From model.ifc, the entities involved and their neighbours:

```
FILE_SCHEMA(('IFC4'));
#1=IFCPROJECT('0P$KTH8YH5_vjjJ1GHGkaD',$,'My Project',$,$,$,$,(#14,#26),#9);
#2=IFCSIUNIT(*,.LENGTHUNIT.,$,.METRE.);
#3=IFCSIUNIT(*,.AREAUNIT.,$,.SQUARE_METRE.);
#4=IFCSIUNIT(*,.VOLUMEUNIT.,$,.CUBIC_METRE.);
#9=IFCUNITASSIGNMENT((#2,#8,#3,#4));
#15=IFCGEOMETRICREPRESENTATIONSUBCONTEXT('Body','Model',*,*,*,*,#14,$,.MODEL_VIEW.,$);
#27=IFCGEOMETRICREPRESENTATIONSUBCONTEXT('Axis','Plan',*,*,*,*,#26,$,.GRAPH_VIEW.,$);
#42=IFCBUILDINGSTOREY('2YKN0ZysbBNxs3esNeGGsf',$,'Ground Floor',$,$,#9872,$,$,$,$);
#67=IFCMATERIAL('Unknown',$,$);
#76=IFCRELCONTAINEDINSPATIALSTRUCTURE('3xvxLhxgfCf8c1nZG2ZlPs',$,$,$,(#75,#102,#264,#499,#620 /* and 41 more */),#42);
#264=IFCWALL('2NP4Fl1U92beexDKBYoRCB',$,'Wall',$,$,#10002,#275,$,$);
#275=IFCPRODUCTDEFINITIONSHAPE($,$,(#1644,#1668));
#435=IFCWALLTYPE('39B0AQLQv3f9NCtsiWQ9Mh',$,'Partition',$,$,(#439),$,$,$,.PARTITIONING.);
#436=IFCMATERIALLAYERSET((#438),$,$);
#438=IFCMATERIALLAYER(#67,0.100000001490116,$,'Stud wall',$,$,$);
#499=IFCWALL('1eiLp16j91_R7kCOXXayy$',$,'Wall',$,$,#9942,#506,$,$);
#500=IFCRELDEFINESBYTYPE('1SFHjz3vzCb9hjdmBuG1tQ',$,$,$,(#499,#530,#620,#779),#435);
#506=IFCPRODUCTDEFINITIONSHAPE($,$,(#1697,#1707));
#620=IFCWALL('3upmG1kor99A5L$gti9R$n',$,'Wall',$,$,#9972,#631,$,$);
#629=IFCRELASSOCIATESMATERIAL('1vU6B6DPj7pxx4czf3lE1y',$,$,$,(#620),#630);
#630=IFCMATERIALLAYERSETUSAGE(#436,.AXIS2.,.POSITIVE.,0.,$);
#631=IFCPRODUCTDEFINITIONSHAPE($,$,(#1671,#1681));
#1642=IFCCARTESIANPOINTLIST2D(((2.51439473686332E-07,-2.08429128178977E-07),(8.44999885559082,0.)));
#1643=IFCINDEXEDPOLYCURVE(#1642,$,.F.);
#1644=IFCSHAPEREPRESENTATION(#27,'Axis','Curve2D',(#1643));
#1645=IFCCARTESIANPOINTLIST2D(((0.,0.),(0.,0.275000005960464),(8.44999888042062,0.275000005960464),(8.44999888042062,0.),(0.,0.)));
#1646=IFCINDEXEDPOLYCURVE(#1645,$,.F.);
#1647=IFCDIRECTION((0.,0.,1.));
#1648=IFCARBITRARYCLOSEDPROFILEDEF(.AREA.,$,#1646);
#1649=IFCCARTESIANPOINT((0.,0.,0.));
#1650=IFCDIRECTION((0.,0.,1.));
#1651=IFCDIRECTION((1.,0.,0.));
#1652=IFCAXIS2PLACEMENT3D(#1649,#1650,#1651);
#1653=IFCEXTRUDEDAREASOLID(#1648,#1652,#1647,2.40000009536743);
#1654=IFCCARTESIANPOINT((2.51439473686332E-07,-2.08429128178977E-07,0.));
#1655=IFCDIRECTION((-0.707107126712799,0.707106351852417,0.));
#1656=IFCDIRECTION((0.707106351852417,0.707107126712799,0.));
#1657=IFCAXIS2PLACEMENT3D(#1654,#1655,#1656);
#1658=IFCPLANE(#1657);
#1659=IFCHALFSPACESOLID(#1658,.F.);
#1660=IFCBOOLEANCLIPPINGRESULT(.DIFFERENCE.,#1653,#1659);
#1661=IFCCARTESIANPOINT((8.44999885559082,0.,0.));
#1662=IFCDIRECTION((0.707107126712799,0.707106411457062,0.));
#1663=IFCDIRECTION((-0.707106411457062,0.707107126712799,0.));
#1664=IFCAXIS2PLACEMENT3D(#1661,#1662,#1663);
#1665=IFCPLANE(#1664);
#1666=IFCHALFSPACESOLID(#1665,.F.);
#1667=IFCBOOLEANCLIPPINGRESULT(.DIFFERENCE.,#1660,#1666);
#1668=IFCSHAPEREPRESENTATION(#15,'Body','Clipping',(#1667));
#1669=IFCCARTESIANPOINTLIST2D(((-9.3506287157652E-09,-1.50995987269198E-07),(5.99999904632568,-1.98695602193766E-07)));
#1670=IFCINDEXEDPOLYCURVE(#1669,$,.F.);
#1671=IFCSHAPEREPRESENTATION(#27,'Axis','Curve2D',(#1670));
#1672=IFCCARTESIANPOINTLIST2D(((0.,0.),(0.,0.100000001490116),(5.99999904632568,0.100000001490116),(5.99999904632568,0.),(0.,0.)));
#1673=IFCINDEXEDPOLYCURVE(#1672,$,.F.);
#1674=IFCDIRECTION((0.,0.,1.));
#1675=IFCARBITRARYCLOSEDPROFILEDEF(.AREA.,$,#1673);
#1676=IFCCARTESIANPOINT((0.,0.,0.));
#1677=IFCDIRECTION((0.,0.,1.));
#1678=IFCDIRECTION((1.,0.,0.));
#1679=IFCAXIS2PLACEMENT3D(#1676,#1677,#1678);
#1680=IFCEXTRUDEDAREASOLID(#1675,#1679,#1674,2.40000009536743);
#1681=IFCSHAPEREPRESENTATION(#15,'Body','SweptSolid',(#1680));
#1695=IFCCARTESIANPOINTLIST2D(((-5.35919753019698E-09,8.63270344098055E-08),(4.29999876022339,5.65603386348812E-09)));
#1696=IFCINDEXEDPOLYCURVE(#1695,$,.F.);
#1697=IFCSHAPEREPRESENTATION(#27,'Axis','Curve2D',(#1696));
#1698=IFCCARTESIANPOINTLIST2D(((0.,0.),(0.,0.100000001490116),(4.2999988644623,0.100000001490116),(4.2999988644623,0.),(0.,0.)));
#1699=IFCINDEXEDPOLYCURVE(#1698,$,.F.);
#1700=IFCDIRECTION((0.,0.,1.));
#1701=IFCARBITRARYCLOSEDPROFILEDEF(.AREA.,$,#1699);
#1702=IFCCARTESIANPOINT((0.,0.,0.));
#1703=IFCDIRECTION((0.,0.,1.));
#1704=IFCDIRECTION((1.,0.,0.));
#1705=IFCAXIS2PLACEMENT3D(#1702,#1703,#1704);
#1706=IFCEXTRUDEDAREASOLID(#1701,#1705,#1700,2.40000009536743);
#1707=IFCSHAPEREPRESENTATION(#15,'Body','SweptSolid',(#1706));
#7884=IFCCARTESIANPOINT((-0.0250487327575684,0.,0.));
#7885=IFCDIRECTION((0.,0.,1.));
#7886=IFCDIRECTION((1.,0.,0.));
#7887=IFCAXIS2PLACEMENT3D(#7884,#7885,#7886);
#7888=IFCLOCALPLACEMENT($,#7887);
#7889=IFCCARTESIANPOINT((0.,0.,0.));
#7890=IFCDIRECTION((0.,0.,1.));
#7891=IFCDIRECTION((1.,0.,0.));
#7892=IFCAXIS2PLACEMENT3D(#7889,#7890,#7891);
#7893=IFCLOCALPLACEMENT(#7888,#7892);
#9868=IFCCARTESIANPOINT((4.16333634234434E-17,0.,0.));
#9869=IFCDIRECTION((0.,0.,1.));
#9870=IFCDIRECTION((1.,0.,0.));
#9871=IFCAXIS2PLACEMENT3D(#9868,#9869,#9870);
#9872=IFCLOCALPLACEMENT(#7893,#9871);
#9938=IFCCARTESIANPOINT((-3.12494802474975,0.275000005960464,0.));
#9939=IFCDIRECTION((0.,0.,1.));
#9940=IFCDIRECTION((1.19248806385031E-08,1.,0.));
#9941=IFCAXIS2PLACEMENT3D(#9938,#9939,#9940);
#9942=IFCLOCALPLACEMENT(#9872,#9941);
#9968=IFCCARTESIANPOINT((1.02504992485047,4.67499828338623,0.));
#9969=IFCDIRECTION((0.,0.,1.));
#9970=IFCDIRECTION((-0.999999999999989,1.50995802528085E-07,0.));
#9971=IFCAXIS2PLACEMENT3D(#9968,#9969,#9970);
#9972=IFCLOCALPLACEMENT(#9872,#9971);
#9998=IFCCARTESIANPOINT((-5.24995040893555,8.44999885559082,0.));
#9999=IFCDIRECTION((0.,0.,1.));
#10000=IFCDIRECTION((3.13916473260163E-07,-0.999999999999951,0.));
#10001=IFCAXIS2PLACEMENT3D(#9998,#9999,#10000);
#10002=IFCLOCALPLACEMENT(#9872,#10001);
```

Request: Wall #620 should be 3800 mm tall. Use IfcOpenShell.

```python
import ifcopenshell
import ifcopenshell.geom
import ifcopenshell.util.representation
import ifcopenshell.util.shape
import ifcopenshell.util.unit

model = ifcopenshell.open("model.ifc")
unit_scale = ifcopenshell.util.unit.calculate_unit_scale(model)
settings = ifcopenshell.geom.settings()


def volume(element):
    """Net volume in cubic metres, openings subtracted."""
    shape = ifcopenshell.geom.create_shape(settings, element)
    return ifcopenshell.util.shape.get_volume(shape.geometry)


wall = model.by_id(620)
before = volume(wall)

body = ifcopenshell.util.representation.get_representation(wall, "Model", "Body")
solid = body.Items[0]
old_height = solid.Depth
solid.Depth = 3.8 / unit_scale
after = volume(wall)

print(f"height {old_height:g} -> {solid.Depth:g}, volume {before:.3f} -> {after:.3f} m3")

model.write("model-out.ifc")
```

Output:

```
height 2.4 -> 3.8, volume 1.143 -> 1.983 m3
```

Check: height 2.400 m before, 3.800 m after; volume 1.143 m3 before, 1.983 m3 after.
